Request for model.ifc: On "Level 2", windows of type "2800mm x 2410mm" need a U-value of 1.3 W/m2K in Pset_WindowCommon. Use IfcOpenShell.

First a look at what the model holds.

```python
import ifcopenshell
import ifcopenshell.util.element

model = ifcopenshell.open("model.ifc")
print(model.schema)
storey = next(s for s in model.by_type("IfcBuildingStorey") if s.Name == "Level 2")
windows = [e for e in ifcopenshell.util.element.get_decomposition(storey) if e.is_a("IfcWindow")]
seen = {}
for e in windows:
    element_type = ifcopenshell.util.element.get_type(e)
    key = (element_type.Name if element_type != e and element_type else None, ifcopenshell.util.element.get_pset(e, "Pset_WindowCommon", "ThermalTransmittance"))
    seen[key] = seen.get(key, 0) + 1
for (name, value), count in sorted(seen.items(), key=str):
    print(count, "x", name, "|", value)
```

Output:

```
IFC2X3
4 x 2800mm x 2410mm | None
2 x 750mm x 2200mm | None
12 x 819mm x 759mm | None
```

```python
import ifcopenshell
import ifcopenshell.api.pset
import ifcopenshell.util.element

model = ifcopenshell.open("model.ifc")

storey = next(s for s in model.by_type("IfcBuildingStorey") if s.Name == "Level 2")
windows = [e for e in ifcopenshell.util.element.get_decomposition(storey) if e.is_a("IfcWindow")]

count = 0
for e in windows:
    element_type = ifcopenshell.util.element.get_type(e)
    if element_type in (None, e) or element_type.Name != "2800mm x 2410mm":
        continue
    # add_pset returns the element's existing set when there is one.
    pset = ifcopenshell.api.pset.add_pset(model, product=e, name="Pset_WindowCommon")
    ifcopenshell.api.pset.edit_pset(model, pset=pset, properties={"ThermalTransmittance": 1.3})
    count += 1

print(count, "windows updated")

model.write("model_edited.ifc")
```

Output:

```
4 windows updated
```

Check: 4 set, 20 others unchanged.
